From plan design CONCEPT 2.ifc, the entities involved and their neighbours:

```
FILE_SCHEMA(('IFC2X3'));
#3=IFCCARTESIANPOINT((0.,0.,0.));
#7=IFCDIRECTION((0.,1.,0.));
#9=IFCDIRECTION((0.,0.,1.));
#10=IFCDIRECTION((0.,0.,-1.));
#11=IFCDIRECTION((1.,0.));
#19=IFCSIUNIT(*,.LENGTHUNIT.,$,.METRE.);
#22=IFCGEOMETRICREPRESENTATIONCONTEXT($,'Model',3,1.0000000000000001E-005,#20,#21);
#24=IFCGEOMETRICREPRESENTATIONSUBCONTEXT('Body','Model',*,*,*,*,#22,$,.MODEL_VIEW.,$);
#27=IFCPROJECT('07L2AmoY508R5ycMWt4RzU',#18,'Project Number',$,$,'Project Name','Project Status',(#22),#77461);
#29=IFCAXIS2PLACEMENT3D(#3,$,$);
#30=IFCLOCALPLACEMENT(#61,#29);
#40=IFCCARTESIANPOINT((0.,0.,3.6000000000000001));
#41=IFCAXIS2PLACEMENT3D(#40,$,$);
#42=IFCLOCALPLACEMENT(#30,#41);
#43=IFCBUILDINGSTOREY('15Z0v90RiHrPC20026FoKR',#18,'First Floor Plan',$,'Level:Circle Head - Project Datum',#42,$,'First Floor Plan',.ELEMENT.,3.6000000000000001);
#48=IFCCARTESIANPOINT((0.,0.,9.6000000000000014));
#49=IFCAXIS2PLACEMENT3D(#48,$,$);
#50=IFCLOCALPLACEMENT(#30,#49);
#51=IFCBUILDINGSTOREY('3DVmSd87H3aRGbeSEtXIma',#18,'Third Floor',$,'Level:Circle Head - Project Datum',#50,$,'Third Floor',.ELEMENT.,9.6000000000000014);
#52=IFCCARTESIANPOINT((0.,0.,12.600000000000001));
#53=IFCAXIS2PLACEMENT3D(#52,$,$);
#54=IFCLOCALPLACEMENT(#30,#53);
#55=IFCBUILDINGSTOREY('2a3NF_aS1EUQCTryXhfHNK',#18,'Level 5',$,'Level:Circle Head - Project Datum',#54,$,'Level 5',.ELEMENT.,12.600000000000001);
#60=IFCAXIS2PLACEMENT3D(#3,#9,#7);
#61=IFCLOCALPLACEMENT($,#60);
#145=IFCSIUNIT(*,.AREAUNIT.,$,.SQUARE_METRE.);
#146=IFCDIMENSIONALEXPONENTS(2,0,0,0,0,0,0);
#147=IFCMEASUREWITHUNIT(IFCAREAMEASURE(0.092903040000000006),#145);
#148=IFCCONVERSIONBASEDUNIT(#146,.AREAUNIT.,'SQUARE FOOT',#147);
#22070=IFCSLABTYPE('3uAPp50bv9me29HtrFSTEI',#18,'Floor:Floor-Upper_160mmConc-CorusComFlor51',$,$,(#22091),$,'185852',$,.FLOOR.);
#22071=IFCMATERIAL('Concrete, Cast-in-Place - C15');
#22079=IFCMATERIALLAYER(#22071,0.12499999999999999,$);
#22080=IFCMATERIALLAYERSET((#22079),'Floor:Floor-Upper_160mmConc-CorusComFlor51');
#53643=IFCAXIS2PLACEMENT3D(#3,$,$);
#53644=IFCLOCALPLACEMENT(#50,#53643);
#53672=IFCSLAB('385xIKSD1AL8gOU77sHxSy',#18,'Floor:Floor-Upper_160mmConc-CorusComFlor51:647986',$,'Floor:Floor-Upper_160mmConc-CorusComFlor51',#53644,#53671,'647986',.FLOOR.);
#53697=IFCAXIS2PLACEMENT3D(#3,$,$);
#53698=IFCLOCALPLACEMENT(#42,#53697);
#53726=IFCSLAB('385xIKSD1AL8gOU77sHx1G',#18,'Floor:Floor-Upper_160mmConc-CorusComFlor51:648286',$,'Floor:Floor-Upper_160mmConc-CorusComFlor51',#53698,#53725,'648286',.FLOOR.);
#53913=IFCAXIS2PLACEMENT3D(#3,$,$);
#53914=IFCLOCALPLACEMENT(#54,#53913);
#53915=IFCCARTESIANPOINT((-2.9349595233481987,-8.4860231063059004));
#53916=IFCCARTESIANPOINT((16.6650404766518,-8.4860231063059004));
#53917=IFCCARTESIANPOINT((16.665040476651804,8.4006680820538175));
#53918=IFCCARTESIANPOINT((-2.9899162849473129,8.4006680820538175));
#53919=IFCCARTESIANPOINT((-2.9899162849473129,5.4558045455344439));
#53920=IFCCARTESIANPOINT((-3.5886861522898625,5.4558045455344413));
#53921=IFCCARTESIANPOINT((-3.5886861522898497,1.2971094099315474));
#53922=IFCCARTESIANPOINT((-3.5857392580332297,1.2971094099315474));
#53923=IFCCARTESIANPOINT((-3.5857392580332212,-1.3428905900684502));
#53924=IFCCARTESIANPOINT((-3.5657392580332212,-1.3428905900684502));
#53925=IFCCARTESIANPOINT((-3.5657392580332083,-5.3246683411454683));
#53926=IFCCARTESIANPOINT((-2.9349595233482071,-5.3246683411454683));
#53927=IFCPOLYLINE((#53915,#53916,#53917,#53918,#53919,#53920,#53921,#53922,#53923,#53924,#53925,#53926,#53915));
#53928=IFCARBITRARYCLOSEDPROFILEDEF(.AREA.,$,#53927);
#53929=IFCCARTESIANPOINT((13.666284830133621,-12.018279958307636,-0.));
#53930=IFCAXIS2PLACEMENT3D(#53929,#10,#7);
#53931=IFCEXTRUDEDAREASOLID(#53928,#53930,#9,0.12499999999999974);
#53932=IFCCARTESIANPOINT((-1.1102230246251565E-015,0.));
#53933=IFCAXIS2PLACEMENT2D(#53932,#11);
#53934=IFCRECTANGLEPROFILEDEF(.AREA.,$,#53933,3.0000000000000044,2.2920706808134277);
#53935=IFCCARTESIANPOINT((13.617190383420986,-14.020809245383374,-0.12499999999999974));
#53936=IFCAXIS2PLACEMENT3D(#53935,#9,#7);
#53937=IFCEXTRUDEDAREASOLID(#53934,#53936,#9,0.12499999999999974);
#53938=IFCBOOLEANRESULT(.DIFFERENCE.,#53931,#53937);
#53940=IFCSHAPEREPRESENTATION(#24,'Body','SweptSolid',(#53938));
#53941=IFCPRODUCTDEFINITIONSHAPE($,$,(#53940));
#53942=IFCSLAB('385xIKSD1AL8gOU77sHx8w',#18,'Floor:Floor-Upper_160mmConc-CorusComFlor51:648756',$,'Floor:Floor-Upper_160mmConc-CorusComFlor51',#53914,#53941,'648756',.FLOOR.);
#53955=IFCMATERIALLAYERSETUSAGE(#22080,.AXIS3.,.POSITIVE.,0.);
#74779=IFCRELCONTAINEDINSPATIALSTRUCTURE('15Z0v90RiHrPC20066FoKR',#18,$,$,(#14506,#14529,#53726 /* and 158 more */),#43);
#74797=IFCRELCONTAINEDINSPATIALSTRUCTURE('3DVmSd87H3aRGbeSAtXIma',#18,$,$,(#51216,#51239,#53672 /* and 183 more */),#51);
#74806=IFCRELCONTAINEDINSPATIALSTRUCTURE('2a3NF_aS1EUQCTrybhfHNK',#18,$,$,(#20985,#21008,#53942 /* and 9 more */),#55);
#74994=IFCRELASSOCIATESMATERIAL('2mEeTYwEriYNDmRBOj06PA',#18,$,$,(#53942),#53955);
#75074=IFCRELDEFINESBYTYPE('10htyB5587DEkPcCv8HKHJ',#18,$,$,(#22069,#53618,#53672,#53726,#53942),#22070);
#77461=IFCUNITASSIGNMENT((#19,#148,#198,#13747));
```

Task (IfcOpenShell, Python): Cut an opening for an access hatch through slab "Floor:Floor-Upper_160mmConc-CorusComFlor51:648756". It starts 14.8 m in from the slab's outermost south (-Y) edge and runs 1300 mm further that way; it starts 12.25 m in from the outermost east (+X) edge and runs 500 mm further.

```python
import numpy as np
import ifcopenshell
import ifcopenshell.api.feature
import ifcopenshell.api.geometry
import ifcopenshell.api.root
import ifcopenshell.geom
import ifcopenshell.util.placement
import ifcopenshell.util.representation
import ifcopenshell.util.shape
import ifcopenshell.util.unit

model = ifcopenshell.open("plan design CONCEPT 2.ifc")
unit_scale = ifcopenshell.util.unit.calculate_unit_scale(model)
settings = ifcopenshell.geom.settings()


def volume(element):
    """Net volume in cubic metres, openings subtracted."""
    shape = ifcopenshell.geom.create_shape(settings, element)
    return ifcopenshell.util.shape.get_volume(shape.geometry)


slab = model.by_id(53942)
before = volume(slab)

# Extent in the slab's own axes, in metres. The edges named are its -X and -Y sides.
slab_shape = ifcopenshell.geom.create_shape(settings, slab)
vertices = ifcopenshell.util.shape.get_vertices(slab_shape.geometry)
x_min, y_min, bottom = vertices.min(axis=0)
top = vertices[:, 2].max()

opening = ifcopenshell.api.root.create_entity(model, ifc_class="IfcOpeningElement", name="Access hatch opening")
context = ifcopenshell.util.representation.get_context(model, "Model", "Body", "MODEL_VIEW")
width, depth = 1.3, 0.5
outline = [(0.0, 0.0), (width, 0.0), (width, depth), (0.0, depth), (0.0, 0.0)]
# Overshoot both faces by 50 mm so the cut is clean.
shape = ifcopenshell.api.geometry.add_slab_representation(
    model, context=context, depth=top - bottom + 0.1, polyline=outline
)
ifcopenshell.api.geometry.assign_representation(model, product=opening, representation=shape)

matrix = ifcopenshell.util.placement.get_local_placement(slab.ObjectPlacement)
matrix[:, 3] = matrix @ np.append(np.array([x_min + 14.8, y_min + 12.25, bottom - 0.05]) / unit_scale, 1.0)
ifcopenshell.api.geometry.edit_object_placement(model, product=opening, matrix=matrix, is_si=False)
ifcopenshell.api.feature.add_feature(model, feature=opening, element=slab)

after = volume(slab)

print(f"slab volume {before:.3f} -> {after:.3f} m3")

model.write("plan design CONCEPT 2-out.ifc")
```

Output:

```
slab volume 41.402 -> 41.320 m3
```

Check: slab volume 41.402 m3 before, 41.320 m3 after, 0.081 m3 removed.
